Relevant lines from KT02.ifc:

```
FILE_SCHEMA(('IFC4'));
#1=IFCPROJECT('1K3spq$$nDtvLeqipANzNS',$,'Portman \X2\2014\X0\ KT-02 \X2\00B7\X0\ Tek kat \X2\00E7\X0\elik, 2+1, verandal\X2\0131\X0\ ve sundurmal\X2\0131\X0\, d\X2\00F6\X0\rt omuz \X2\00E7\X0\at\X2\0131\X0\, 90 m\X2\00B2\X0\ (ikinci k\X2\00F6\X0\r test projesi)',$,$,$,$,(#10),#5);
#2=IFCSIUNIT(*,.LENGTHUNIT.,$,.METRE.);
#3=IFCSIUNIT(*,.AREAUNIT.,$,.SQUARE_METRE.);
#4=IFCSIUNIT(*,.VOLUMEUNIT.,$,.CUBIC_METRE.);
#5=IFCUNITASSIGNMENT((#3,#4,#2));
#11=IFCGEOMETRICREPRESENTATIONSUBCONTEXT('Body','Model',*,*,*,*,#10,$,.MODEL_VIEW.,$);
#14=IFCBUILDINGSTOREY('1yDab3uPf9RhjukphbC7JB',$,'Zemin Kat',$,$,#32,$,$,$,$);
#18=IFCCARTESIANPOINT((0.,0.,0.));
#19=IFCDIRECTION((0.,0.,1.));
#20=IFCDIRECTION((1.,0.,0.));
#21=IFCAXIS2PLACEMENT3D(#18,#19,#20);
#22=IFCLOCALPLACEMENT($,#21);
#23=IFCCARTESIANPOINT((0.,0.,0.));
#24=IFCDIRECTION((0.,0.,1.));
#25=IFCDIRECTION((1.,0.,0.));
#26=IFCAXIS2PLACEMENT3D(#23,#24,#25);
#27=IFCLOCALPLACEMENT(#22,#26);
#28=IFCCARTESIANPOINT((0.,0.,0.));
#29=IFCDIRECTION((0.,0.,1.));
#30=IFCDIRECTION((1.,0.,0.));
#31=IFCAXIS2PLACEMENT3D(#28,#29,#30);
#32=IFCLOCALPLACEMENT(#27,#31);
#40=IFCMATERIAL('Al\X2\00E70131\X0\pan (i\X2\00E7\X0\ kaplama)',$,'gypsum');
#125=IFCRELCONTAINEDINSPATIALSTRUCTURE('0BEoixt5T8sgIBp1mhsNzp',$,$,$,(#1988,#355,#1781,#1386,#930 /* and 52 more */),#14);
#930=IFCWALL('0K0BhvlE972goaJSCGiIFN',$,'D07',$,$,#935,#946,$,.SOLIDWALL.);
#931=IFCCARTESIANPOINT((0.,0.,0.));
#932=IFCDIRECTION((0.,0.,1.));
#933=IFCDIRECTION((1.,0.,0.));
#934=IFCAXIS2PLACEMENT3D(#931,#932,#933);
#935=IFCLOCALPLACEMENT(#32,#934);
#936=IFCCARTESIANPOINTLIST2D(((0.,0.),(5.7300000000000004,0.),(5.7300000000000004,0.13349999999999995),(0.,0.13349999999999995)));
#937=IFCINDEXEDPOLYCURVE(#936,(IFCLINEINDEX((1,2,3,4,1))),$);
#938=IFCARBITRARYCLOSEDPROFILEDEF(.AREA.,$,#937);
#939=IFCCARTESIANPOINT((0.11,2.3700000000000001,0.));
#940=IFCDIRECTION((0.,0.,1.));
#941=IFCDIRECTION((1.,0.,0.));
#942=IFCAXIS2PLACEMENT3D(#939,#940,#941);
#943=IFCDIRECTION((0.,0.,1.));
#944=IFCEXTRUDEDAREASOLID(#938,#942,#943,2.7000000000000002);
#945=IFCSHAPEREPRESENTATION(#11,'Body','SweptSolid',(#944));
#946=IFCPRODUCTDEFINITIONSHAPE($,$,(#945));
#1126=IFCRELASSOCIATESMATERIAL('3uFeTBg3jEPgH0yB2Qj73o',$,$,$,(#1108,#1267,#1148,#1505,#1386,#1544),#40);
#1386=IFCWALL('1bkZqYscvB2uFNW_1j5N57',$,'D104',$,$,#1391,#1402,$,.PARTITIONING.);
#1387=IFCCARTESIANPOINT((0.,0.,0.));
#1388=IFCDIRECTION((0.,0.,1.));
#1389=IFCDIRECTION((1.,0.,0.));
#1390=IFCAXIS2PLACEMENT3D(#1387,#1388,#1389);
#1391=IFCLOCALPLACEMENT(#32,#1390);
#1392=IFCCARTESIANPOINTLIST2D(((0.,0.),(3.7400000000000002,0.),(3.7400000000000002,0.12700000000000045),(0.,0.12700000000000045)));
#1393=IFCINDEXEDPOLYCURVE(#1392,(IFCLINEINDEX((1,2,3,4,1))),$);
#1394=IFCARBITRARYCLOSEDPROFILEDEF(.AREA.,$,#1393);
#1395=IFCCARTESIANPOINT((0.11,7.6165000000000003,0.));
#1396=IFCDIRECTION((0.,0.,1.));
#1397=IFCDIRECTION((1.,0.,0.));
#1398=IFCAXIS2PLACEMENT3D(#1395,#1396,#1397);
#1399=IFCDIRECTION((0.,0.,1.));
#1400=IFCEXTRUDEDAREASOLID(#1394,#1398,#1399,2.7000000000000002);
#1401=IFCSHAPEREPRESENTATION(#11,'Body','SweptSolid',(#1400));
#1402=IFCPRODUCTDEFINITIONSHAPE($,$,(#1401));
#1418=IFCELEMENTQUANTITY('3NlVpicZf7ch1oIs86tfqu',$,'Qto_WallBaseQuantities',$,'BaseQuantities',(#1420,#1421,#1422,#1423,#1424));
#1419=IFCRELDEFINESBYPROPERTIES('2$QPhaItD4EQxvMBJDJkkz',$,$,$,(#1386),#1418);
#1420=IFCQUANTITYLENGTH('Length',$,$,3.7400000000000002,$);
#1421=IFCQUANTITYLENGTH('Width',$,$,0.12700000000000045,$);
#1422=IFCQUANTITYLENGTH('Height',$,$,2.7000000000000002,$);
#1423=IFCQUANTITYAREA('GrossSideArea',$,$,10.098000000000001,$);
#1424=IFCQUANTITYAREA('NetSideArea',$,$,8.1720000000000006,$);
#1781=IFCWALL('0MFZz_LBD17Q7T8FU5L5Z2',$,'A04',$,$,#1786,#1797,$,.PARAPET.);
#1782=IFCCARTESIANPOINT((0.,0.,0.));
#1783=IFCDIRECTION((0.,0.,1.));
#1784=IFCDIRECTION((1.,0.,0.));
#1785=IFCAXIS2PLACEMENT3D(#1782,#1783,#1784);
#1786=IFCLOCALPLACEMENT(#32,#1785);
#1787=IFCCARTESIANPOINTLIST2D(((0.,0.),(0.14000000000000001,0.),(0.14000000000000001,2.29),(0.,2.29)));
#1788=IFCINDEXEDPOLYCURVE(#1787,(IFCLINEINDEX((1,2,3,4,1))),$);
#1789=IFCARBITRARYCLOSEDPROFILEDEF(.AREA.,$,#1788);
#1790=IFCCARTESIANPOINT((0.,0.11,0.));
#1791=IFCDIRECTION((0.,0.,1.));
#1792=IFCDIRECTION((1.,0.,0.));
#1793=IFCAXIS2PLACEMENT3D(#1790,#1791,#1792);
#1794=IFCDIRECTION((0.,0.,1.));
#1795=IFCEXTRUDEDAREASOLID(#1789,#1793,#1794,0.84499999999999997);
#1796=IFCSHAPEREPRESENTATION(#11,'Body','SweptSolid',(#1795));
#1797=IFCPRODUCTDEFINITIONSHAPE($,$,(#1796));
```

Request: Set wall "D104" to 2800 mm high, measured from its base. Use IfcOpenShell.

```python
import ifcopenshell
import ifcopenshell.api.pset
import ifcopenshell.geom
import ifcopenshell.util.element
import ifcopenshell.util.representation
import ifcopenshell.util.shape
import ifcopenshell.util.unit

model = ifcopenshell.open("KT02.ifc")
unit_scale = ifcopenshell.util.unit.calculate_unit_scale(model)
area_scale = ifcopenshell.util.unit.calculate_unit_scale(model, "AREAUNIT")
settings = ifcopenshell.geom.settings()


def volume(element):
    """Net volume in cubic metres, openings subtracted."""
    shape = ifcopenshell.geom.create_shape(settings, element)
    return ifcopenshell.util.shape.get_volume(shape.geometry)


wall = model.by_id(1386)
before = volume(wall)

body = ifcopenshell.util.representation.get_representation(wall, "Model", "Body")
solid = body.Items[0]
old_height = solid.Depth
solid.Depth = 2.8
after = volume(wall)
thickness = 0.127  # wall thickness in metres

# Update the stored height, areas and volumes.
qto = model.by_id(ifcopenshell.util.element.get_pset(wall, "Qto_WallBaseQuantities", should_inherit=False)["id"])
ifcopenshell.api.pset.edit_qto(model, qto=qto, properties={
    "Height": solid.Depth,
    "GrossSideArea": ifcopenshell.util.element.get_pset(wall, "Qto_WallBaseQuantities", "GrossSideArea") * solid.Depth / old_height,
    "NetSideArea": after / thickness / area_scale,
})

print(f"height {old_height:g} -> {solid.Depth:g}, volume {before:.3f} -> {after:.3f} m3")

model.write("KT02_updated.ifc")
```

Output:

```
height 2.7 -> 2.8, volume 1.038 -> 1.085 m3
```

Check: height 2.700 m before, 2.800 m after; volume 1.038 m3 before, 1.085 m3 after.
